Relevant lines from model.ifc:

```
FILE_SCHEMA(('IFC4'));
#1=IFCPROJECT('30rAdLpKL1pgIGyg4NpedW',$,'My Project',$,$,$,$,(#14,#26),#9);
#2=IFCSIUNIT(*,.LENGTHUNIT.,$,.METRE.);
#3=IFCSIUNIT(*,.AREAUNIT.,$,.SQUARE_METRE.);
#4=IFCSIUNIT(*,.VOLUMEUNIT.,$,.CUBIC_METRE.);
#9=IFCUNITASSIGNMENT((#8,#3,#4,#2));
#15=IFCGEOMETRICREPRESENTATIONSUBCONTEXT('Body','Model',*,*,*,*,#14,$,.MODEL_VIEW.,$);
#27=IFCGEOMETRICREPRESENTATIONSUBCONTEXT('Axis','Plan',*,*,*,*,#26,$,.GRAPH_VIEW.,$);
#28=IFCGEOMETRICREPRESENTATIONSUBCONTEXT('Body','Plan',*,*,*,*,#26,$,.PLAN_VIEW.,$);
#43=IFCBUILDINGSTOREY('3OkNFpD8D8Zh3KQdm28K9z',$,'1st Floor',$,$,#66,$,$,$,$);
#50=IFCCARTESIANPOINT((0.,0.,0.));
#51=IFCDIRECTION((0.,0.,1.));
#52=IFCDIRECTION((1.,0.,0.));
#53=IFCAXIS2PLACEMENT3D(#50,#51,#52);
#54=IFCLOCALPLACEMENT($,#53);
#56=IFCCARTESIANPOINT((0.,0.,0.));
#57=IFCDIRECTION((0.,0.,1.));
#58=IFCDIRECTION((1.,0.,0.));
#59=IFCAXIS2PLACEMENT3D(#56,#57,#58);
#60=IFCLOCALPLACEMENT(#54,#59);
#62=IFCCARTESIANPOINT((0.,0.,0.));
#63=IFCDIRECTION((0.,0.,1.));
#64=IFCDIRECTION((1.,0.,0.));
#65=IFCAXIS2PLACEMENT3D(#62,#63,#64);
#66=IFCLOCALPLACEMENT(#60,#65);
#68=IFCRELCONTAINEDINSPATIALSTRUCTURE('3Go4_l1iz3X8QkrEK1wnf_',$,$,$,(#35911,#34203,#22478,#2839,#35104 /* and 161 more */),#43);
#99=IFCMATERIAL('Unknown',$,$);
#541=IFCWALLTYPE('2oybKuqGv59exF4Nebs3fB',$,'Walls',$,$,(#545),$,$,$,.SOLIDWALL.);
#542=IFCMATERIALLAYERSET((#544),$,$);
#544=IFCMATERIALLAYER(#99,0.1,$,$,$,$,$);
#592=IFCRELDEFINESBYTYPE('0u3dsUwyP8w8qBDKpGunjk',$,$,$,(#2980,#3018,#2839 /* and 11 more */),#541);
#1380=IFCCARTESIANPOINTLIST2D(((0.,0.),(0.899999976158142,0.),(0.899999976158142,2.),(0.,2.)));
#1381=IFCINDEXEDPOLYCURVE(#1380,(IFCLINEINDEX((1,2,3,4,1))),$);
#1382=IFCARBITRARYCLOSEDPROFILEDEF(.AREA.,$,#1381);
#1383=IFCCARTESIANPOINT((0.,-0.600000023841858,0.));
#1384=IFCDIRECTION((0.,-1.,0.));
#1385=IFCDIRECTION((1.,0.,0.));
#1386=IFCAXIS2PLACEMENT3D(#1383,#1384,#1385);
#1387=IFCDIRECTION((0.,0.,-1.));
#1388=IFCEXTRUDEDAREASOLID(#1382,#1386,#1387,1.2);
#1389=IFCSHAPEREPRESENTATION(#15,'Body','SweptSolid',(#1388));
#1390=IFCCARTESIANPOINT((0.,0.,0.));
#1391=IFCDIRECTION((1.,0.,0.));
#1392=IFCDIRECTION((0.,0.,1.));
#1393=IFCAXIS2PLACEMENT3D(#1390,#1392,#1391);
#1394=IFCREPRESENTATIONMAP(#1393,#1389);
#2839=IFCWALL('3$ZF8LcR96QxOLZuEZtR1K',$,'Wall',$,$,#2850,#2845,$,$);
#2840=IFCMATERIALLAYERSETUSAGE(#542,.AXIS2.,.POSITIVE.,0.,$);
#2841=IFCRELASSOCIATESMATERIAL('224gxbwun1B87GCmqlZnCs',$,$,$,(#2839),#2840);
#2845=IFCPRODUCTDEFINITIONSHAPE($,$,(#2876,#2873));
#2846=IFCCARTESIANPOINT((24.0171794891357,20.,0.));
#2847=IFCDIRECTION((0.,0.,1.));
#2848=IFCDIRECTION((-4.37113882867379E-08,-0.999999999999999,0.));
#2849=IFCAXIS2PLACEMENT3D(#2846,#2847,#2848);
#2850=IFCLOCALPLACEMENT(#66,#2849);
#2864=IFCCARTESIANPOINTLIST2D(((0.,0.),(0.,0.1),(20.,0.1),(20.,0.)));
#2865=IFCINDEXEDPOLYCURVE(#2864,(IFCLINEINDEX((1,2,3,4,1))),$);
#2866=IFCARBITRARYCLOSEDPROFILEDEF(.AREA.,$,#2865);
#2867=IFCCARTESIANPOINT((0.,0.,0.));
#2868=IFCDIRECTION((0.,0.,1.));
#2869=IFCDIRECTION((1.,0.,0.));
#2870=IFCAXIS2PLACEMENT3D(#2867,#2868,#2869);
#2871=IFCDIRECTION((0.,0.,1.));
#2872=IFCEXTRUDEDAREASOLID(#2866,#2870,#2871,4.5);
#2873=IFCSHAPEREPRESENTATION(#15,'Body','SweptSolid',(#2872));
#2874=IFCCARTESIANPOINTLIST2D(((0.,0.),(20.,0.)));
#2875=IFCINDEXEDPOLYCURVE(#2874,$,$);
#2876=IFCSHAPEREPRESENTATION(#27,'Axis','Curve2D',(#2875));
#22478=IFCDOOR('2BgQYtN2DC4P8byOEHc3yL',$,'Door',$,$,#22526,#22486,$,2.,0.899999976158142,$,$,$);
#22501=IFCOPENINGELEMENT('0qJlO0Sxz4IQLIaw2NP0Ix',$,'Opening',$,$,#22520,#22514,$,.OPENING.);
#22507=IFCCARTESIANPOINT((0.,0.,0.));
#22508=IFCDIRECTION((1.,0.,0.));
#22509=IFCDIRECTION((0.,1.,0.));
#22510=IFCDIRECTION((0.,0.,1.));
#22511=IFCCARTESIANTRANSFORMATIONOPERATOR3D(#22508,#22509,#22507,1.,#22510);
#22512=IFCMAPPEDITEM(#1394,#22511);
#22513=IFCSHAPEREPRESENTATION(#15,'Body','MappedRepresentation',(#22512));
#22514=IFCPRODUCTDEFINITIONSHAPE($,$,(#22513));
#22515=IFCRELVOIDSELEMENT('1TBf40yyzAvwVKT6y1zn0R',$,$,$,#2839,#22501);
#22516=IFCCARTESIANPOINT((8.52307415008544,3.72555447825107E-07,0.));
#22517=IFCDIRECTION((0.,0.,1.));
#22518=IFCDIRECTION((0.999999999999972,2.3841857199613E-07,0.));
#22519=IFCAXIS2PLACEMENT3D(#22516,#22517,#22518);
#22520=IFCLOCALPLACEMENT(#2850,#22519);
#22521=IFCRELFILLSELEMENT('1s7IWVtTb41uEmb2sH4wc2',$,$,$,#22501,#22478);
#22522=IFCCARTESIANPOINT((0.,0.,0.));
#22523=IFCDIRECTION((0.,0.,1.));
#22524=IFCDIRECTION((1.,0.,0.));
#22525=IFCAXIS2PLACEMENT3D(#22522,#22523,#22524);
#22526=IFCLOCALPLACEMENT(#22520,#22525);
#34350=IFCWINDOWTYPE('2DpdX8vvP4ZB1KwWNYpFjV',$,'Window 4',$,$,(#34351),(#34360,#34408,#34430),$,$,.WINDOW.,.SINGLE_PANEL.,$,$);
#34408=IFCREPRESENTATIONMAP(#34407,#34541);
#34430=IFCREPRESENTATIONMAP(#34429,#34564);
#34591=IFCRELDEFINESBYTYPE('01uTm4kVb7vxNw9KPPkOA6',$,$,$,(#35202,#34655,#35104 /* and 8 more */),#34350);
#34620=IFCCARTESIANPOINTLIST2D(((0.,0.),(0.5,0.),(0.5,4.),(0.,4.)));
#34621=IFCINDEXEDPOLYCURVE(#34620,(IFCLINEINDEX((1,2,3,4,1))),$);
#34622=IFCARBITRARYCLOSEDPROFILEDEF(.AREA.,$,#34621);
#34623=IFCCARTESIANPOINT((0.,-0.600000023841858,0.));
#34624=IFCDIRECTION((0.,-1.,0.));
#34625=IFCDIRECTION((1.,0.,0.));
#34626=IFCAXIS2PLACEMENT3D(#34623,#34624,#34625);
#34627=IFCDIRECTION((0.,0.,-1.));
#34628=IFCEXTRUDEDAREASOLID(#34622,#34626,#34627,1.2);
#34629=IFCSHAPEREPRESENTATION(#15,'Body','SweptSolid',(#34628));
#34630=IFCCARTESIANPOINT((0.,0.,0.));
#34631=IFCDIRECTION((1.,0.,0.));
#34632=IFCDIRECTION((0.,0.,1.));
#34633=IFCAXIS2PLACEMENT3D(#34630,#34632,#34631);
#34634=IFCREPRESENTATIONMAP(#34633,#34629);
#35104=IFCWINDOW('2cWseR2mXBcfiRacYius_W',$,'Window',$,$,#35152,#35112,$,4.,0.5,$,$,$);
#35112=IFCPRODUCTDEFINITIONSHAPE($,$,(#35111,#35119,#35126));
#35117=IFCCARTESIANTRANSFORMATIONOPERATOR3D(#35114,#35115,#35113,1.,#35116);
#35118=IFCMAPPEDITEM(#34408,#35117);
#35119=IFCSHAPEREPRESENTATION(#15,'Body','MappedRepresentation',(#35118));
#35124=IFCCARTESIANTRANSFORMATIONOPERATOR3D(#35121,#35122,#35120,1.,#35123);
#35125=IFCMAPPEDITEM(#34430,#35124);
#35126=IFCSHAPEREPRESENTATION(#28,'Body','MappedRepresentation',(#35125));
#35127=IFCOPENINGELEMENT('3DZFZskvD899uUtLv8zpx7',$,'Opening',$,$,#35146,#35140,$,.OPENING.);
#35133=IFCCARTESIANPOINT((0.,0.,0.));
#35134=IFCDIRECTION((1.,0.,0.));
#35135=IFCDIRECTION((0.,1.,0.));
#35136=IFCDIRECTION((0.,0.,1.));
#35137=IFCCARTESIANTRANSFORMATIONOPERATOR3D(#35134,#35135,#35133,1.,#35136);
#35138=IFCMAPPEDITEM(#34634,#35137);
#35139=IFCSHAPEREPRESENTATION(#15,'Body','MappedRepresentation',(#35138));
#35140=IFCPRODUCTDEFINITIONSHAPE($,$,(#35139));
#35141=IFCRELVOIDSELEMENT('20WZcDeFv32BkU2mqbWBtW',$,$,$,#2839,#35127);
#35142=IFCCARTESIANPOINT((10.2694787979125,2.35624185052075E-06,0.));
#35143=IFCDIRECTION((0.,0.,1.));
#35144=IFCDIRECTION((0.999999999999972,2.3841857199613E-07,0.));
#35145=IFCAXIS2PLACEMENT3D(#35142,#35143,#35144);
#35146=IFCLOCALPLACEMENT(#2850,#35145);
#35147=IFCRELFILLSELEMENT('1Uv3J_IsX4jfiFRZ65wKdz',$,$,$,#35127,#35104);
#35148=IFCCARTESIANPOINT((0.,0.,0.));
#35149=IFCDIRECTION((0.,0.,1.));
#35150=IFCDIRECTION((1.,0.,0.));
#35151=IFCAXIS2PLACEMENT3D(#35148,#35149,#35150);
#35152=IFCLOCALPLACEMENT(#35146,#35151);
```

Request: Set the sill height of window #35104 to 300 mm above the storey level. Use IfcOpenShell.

```python
import numpy as np
import ifcopenshell
import ifcopenshell.api.geometry
import ifcopenshell.geom
import ifcopenshell.util.element
import ifcopenshell.util.placement
import ifcopenshell.util.shape
import ifcopenshell.util.unit

model = ifcopenshell.open("model.ifc")
unit_scale = ifcopenshell.util.unit.calculate_unit_scale(model)

window = model.by_guid("2cWseR2mXBcfiRacYius_W")
opening = window.FillsVoids[0].RelatingOpeningElement
storey = ifcopenshell.util.element.get_container(window, ifc_class="IfcBuildingStorey")
level = ifcopenshell.util.placement.get_local_placement(storey.ObjectPlacement)[2, 3]

# The opening's origin need not be at the sill, so measure its lowest point.
shape = ifcopenshell.geom.create_shape(ifcopenshell.geom.settings(), opening)
bottom = ifcopenshell.util.shape.get_shape_bottom_elevation(shape, shape.geometry) / unit_scale
dz = level + 0.3 / unit_scale - bottom

shift = np.array([0.0, 0.0, dz])
# The window is placed relative to its opening, so it follows when the opening moves.
matrix = ifcopenshell.util.placement.get_local_placement(opening.ObjectPlacement)
matrix[:3, 3] += shift
ifcopenshell.api.geometry.edit_object_placement(
    model, product=opening, matrix=matrix, is_si=False, should_transform_children=True
)

print(f"moved by {dz * unit_scale:+.3f} m")

model.write("model_rev.ifc")
```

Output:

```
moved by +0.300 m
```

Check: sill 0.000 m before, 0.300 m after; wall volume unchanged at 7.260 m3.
